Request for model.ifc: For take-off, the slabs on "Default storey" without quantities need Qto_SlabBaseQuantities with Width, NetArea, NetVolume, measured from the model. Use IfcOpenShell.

First a look at what the model holds.

```python
import ifcopenshell
import ifcopenshell.util.element
import ifcopenshell.util.unit

model = ifcopenshell.open("model.ifc")
print(model.schema)
for unit_type in ("LENGTHUNIT", "AREAUNIT", "VOLUMEUNIT"):
    print(unit_type, ifcopenshell.util.unit.calculate_unit_scale(model, unit_type))
storey = next(s for s in model.by_type("IfcBuildingStorey") if s.Name == "Default storey")
slabs = [e for e in ifcopenshell.util.element.get_decomposition(storey) if e.is_a("IfcSlab")]
for e in sorted(slabs, key=lambda e: e.id()):
    print(e.id(), e.is_a(), e.Name, list(ifcopenshell.util.element.get_psets(e, qtos_only=True)), sep=" | ")
```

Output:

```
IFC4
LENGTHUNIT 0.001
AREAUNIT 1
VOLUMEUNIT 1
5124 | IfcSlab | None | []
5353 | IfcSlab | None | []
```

```python
import ifcopenshell
import ifcopenshell.api.pset
import ifcopenshell.geom
import ifcopenshell.util.element
import ifcopenshell.util.shape
import ifcopenshell.util.unit

model = ifcopenshell.open("model.ifc")
unit_scale = ifcopenshell.util.unit.calculate_unit_scale(model)
area_scale = ifcopenshell.util.unit.calculate_unit_scale(model, "AREAUNIT")
volume_scale = ifcopenshell.util.unit.calculate_unit_scale(model, "VOLUMEUNIT")
settings = ifcopenshell.geom.settings()

storey = next(s for s in model.by_type("IfcBuildingStorey") if s.Name == "Default storey")
slabs = [e for e in ifcopenshell.util.element.get_decomposition(storey) if e.is_a("IfcSlab")]

for e in sorted(slabs, key=lambda e: e.id()):
    if ifcopenshell.util.element.get_psets(e, qtos_only=True, should_inherit=False):
        continue
    # Geometry comes back in metres, in the element's own axes.
    shape = ifcopenshell.geom.create_shape(settings, e)
    values = {
        "Width": ifcopenshell.util.shape.get_z(shape.geometry) / unit_scale,
        "NetArea": ifcopenshell.util.shape.get_footprint_area(shape.geometry) / area_scale,
        "NetVolume": ifcopenshell.util.shape.get_volume(shape.geometry) / volume_scale,
    }
    qto = ifcopenshell.api.pset.add_qto(model, product=e, name="Qto_SlabBaseQuantities")
    ifcopenshell.api.pset.edit_qto(model, qto=qto, properties=values)
    print(e.id(), {k: round(v, 3) for k, v in values.items()})

model.write("model_edited.ifc")
```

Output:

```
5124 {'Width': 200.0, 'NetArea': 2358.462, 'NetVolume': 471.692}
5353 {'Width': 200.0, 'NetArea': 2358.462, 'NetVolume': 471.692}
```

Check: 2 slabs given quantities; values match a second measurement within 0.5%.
